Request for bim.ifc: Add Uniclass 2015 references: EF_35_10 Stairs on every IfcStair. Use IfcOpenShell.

First a look at what the model holds.

```python
import ifcopenshell

model = ifcopenshell.open("bim.ifc")
print(model.schema)
print("classifications:", [c.Name for c in model.by_type("IfcClassification")])
for ifc_class in ("IfcDoor", "IfcRoof", "IfcStair", "IfcWall", "IfcWindow"):
    print(ifc_class, len(model.by_type(ifc_class)))
```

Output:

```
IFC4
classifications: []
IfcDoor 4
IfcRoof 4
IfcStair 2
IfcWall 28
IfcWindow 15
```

```python
import ifcopenshell
import ifcopenshell.api.classification

model = ifcopenshell.open("bim.ifc")

system = ifcopenshell.api.classification.add_classification(model, classification="Uniclass 2015")

codes = {
    "IfcStair": ("EF_35_10", "Stairs"),
}
for ifc_class, (code, name) in codes.items():
    products = model.by_type(ifc_class)
    ifcopenshell.api.classification.add_reference(
        model, products=products, classification=system, identification=code, name=name
    )
    print(code, len(products))

model.write("bim_edited.ifc")
```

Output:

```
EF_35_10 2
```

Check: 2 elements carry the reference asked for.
